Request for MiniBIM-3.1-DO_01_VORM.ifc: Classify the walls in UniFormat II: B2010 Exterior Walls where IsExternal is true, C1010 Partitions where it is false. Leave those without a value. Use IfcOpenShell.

First a look at what the model holds.

```python
import ifcopenshell
import ifcopenshell.util.element

model = ifcopenshell.open("MiniBIM-3.1-DO_01_VORM.ifc")
print(model.schema)
print("classifications:", [c.Name for c in model.by_type("IfcClassification")])
values = [ifcopenshell.util.element.get_pset(e, "Pset_WallCommon", "IsExternal") for e in model.by_type("IfcWall")]
for value in (True, False, None):
    print("IsExternal", value, values.count(value))
```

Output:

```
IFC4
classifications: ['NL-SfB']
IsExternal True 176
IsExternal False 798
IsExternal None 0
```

```python
import ifcopenshell
import ifcopenshell.api.classification
import ifcopenshell.util.element

model = ifcopenshell.open("MiniBIM-3.1-DO_01_VORM.ifc")

system = ifcopenshell.api.classification.add_classification(model, classification="UniFormat II")

walls = model.by_type("IfcWall")
external = {e: ifcopenshell.util.element.get_pset(e, "Pset_WallCommon", "IsExternal") for e in walls}
for flag, code, name in ((True, "B2010", "Exterior Walls"), (False, "C1010", "Partitions")):
    products = [e for e in walls if external[e] is flag]
    ifcopenshell.api.classification.add_reference(
        model, products=products, classification=system, identification=code, name=name
    )
    print(code, len(products))

model.write("MiniBIM-3.1-DO_01_VORM_rev.ifc")
```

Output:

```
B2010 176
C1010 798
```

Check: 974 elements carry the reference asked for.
